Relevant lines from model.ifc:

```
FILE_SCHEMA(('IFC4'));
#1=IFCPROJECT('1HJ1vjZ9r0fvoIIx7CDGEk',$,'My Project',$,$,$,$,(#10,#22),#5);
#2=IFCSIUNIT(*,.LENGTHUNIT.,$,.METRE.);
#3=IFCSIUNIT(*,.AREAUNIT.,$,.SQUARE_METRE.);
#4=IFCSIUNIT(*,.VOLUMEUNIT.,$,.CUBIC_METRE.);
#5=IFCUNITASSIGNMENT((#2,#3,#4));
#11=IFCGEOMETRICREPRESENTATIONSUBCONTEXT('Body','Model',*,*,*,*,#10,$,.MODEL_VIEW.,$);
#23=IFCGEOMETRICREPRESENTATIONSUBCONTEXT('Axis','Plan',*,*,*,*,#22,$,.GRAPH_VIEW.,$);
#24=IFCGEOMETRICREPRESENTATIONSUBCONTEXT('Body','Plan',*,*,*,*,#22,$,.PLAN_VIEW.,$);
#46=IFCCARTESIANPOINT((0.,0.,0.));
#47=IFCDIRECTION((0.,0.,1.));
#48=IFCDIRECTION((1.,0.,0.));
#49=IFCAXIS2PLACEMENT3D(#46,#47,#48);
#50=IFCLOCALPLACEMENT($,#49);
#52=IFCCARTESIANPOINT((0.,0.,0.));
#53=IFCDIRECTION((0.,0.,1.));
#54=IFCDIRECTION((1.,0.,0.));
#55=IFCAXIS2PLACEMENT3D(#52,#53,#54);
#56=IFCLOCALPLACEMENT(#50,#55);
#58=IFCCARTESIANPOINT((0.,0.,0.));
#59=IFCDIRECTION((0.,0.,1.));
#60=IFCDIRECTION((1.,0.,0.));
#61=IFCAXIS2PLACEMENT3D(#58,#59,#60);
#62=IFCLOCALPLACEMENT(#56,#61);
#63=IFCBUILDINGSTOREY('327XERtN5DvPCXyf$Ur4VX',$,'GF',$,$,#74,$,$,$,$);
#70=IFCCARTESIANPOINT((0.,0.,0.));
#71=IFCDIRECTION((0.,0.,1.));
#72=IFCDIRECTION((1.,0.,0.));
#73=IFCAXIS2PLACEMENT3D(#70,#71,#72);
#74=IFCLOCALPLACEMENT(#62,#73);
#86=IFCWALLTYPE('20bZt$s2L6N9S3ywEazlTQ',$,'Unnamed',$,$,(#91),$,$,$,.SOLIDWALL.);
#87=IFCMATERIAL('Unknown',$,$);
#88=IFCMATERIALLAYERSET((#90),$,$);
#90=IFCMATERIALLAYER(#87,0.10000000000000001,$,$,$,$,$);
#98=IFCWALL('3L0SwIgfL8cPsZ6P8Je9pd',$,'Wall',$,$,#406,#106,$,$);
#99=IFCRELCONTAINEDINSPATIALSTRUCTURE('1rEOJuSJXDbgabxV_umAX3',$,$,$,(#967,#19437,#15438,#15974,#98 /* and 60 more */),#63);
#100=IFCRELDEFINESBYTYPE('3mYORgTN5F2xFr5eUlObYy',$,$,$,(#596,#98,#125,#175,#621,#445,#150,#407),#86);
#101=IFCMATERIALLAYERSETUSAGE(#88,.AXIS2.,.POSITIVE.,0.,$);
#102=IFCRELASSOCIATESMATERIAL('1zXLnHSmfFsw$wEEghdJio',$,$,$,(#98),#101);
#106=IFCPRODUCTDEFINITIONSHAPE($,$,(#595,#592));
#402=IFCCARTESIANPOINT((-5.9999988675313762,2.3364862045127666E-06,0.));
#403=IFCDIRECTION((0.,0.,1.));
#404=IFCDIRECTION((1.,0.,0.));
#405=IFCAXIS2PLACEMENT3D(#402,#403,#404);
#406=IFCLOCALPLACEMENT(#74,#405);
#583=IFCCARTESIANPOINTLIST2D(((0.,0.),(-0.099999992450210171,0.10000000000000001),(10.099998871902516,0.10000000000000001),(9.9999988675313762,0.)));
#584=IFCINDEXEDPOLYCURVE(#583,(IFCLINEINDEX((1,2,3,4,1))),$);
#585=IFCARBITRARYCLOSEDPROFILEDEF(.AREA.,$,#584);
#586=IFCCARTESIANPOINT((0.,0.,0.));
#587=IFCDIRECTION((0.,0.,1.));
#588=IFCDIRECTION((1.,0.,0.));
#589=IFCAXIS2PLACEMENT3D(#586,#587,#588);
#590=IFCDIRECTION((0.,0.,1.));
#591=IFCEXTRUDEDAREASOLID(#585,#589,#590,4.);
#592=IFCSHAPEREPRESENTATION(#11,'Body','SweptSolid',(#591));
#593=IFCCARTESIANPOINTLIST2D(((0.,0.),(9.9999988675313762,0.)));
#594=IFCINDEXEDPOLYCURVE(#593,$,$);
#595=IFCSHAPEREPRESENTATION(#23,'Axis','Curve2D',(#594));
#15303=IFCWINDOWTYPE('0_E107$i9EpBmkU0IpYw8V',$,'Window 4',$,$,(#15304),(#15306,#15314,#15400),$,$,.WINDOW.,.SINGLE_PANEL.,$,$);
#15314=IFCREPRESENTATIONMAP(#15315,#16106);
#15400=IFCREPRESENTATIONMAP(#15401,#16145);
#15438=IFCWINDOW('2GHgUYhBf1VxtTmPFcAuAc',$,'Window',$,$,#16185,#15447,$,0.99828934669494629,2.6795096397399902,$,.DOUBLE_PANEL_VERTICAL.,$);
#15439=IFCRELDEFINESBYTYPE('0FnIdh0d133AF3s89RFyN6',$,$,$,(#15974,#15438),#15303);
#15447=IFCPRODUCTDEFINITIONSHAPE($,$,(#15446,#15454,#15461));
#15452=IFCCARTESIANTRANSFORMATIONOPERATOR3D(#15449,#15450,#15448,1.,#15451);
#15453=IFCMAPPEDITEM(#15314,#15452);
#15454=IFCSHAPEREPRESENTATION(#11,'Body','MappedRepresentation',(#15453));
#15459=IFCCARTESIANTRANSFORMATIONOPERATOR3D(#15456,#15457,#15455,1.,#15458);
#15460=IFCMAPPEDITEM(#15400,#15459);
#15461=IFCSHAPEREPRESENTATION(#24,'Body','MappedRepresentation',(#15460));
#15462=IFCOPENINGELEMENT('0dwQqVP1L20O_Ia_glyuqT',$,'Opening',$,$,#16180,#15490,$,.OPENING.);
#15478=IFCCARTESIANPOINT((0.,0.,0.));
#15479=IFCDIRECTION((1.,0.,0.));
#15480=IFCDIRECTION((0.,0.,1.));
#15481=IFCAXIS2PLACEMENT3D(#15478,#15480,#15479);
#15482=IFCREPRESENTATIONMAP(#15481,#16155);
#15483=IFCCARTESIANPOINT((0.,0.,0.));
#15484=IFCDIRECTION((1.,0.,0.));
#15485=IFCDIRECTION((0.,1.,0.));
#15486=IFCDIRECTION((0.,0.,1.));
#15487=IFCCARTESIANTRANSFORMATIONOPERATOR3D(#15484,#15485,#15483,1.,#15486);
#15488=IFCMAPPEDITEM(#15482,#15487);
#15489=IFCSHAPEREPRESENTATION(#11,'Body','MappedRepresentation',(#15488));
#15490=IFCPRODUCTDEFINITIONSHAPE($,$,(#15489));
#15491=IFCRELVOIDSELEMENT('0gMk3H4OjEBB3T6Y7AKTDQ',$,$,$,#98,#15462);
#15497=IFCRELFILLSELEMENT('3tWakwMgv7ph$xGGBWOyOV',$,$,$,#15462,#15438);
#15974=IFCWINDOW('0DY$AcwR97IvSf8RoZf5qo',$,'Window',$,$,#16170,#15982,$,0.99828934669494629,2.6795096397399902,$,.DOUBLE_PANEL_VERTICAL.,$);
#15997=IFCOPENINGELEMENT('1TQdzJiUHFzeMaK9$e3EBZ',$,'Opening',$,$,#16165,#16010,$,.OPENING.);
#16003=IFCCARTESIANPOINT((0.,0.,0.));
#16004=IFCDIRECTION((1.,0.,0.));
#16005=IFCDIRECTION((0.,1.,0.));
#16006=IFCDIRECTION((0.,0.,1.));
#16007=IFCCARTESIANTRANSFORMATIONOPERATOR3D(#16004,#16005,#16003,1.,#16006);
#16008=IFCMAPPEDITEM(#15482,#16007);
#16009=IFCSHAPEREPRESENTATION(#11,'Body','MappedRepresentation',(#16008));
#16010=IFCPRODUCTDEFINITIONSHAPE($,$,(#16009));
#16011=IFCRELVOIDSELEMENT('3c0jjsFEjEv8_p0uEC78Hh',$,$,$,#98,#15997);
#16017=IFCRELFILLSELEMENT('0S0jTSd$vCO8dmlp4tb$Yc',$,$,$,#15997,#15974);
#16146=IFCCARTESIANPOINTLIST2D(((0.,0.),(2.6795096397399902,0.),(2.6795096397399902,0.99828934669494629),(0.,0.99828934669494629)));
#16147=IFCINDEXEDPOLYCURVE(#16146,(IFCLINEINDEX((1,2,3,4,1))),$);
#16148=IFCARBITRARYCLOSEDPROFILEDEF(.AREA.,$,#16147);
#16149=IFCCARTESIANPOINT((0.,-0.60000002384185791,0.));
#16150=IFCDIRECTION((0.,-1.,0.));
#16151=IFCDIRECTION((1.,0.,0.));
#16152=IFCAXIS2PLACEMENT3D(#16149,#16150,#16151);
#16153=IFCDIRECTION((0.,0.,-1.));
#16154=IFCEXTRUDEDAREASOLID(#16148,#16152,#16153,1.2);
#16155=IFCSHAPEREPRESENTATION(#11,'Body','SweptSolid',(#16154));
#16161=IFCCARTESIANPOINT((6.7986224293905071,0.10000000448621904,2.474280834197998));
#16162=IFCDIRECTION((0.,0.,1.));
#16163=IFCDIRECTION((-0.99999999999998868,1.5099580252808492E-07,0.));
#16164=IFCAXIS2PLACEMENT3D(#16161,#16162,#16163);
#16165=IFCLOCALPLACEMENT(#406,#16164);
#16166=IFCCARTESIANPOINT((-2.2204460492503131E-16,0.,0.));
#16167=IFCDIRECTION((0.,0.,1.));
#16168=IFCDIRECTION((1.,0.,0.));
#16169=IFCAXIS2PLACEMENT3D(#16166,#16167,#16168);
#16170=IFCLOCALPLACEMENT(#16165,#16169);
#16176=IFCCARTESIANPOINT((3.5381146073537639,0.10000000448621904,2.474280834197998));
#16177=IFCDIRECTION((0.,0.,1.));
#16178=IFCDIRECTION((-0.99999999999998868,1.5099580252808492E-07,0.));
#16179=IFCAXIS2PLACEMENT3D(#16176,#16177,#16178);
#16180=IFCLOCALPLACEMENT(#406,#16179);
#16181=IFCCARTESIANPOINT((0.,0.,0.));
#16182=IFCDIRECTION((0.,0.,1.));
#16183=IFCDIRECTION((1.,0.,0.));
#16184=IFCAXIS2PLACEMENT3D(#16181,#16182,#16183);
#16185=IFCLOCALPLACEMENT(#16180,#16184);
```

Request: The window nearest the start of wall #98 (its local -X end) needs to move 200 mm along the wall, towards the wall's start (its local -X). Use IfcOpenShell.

```python
import ifcopenshell
import ifcopenshell.api.geometry
import ifcopenshell.util.placement
import ifcopenshell.util.unit

model = ifcopenshell.open("model.ifc")
unit_scale = ifcopenshell.util.unit.calculate_unit_scale(model)

window = model.by_guid("2GHgUYhBf1VxtTmPFcAuAc")
opening = window.FillsVoids[0].RelatingOpeningElement
wall = opening.VoidsElements[0].RelatingBuildingElement

wall_matrix = ifcopenshell.util.placement.get_local_placement(wall.ObjectPlacement)
shift = wall_matrix[:3, 0] * -0.2 / unit_scale
before = ifcopenshell.util.placement.get_local_placement(window.ObjectPlacement)[:3, 3].copy()

# The window is placed relative to its opening, so it follows when the opening moves.
matrix = ifcopenshell.util.placement.get_local_placement(opening.ObjectPlacement)
matrix[:3, 3] += shift
ifcopenshell.api.geometry.edit_object_placement(
    model, product=opening, matrix=matrix, is_si=False, should_transform_children=True
)

after = ifcopenshell.util.placement.get_local_placement(window.ObjectPlacement)[:3, 3]
print("window moved by", (after - before).round(3) + 0.0)

model.write("model-out.ifc")
```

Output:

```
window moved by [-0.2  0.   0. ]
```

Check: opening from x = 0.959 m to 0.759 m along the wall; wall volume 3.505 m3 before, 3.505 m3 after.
